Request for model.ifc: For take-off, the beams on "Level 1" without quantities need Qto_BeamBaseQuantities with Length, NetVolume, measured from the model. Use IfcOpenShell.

First a look at what the model holds.

```python
import ifcopenshell
import ifcopenshell.util.element
import ifcopenshell.util.unit

model = ifcopenshell.open("model.ifc")
print(model.schema)
for unit_type in ("LENGTHUNIT", "AREAUNIT", "VOLUMEUNIT"):
    print(unit_type, ifcopenshell.util.unit.calculate_unit_scale(model, unit_type))
storey = next(s for s in model.by_type("IfcBuildingStorey") if s.Name == "Level 1")
beams = [e for e in ifcopenshell.util.element.get_decomposition(storey) if e.is_a("IfcBeam")]
for e in sorted(beams, key=lambda e: e.id()):
    print(e.id(), e.is_a(), e.Name, list(ifcopenshell.util.element.get_psets(e, qtos_only=True)), sep=" | ")
```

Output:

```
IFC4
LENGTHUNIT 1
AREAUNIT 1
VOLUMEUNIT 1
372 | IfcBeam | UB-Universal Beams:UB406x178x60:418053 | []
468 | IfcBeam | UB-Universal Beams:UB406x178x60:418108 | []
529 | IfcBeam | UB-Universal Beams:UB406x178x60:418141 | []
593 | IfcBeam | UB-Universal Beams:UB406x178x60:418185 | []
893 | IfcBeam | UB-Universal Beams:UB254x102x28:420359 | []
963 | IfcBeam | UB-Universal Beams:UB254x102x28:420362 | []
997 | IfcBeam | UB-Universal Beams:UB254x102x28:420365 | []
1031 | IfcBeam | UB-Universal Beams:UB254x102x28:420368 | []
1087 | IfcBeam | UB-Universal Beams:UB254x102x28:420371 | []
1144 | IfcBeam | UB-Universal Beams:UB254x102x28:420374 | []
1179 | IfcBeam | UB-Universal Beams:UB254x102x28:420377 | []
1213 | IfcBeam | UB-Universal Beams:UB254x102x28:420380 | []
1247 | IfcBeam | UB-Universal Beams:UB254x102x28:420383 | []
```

```python
import ifcopenshell
import ifcopenshell.api.pset
import ifcopenshell.geom
import ifcopenshell.util.element
import ifcopenshell.util.shape
import ifcopenshell.util.unit

model = ifcopenshell.open("model.ifc")
unit_scale = ifcopenshell.util.unit.calculate_unit_scale(model)
volume_scale = ifcopenshell.util.unit.calculate_unit_scale(model, "VOLUMEUNIT")
settings = ifcopenshell.geom.settings()

storey = next(s for s in model.by_type("IfcBuildingStorey") if s.Name == "Level 1")
beams = [e for e in ifcopenshell.util.element.get_decomposition(storey) if e.is_a("IfcBeam")]

for e in sorted(beams, key=lambda e: e.id()):
    if ifcopenshell.util.element.get_psets(e, qtos_only=True, should_inherit=False):
        continue
    # Geometry comes back in metres, in the element's own axes.
    shape = ifcopenshell.geom.create_shape(settings, e)
    values = {
        "Length": ifcopenshell.util.shape.get_max_xyz(shape.geometry) / unit_scale,
        "NetVolume": ifcopenshell.util.shape.get_volume(shape.geometry) / volume_scale,
    }
    qto = ifcopenshell.api.pset.add_qto(model, product=e, name="Qto_BeamBaseQuantities")
    ifcopenshell.api.pset.edit_qto(model, qto=qto, properties=values)
    print(e.id(), {k: round(v, 3) for k, v in values.items()})

model.write("model_v2.ifc")
```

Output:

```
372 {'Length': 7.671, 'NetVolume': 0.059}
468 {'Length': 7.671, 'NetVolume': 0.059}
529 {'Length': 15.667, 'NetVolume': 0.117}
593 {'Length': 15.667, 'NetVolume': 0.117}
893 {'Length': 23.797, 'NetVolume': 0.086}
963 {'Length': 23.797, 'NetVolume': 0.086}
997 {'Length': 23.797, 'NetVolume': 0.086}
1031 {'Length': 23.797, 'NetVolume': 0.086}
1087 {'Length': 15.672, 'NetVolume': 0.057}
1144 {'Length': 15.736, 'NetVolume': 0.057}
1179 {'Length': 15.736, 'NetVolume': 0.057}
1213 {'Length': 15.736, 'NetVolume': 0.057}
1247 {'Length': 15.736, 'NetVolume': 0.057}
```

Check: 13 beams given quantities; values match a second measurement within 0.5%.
